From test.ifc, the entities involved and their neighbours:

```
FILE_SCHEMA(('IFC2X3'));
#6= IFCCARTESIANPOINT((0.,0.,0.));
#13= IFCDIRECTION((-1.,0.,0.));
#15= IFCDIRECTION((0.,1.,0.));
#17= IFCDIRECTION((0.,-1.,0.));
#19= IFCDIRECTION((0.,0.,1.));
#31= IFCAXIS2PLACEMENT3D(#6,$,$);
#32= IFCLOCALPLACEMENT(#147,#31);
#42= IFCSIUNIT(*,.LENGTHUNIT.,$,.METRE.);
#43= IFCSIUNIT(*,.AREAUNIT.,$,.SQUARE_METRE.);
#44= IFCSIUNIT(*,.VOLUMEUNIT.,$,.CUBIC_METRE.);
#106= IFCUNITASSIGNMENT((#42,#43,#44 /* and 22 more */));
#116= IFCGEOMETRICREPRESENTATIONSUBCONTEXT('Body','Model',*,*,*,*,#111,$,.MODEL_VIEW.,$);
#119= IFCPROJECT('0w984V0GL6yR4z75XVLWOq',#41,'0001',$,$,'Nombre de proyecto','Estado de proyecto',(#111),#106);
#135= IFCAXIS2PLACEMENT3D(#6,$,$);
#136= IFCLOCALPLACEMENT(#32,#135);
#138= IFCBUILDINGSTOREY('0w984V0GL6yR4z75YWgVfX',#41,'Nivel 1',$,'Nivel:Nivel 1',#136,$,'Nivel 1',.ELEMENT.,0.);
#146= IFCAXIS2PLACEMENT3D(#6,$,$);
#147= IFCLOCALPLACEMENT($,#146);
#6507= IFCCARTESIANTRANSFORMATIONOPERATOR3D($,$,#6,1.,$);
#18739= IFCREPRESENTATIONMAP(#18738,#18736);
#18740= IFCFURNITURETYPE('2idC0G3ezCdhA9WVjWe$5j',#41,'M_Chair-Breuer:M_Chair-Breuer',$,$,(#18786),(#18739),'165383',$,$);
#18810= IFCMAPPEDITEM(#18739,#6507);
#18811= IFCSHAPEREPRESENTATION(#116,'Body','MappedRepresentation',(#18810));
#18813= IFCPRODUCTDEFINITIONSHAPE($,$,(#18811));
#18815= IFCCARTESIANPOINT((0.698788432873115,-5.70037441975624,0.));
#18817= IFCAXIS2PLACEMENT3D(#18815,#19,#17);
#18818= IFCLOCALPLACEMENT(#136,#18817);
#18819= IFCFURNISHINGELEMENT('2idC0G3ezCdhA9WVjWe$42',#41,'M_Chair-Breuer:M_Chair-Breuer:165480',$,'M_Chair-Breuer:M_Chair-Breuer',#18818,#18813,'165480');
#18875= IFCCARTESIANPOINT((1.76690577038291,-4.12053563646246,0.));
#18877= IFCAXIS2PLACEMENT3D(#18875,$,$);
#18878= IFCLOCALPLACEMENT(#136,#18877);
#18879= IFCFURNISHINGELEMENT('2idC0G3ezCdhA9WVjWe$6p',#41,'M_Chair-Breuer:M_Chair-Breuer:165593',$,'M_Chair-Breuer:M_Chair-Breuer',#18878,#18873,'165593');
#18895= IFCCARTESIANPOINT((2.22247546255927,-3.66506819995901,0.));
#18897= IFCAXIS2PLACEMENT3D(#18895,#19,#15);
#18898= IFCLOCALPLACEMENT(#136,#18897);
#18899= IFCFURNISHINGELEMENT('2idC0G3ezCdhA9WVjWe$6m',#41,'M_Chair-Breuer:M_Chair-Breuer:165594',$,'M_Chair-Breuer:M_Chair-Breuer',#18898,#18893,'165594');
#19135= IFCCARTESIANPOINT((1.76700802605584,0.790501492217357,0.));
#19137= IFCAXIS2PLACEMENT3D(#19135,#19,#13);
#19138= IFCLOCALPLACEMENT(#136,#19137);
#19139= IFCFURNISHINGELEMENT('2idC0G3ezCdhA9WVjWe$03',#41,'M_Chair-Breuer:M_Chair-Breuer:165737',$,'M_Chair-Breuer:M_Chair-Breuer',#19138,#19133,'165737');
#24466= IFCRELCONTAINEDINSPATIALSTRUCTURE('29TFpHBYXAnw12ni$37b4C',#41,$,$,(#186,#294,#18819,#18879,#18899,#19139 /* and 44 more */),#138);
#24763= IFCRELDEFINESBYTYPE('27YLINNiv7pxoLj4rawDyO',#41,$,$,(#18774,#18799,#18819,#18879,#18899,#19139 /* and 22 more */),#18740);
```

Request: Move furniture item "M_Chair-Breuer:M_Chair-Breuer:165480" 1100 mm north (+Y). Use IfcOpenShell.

```python
import ifcopenshell
import ifcopenshell.api.geometry
import ifcopenshell.util.placement
import ifcopenshell.util.unit

model = ifcopenshell.open("test.ifc")
unit_scale = ifcopenshell.util.unit.calculate_unit_scale(model)

item = model.by_guid("2idC0G3ezCdhA9WVjWe$42")
matrix = ifcopenshell.util.placement.get_local_placement(item.ObjectPlacement)
matrix[1, 3] += 1.1 / unit_scale
ifcopenshell.api.geometry.edit_object_placement(model, product=item, matrix=matrix, is_si=False)

print(ifcopenshell.util.placement.get_local_placement(item.ObjectPlacement).round(3) + 0.0)

model.write("test_edited.ifc")
```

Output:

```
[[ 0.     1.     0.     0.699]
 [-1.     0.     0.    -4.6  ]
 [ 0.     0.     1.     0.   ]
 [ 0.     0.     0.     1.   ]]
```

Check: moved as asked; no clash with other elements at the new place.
